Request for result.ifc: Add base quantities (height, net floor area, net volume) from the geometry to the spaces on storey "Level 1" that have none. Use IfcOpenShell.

First a look at what the model holds.

```python
import ifcopenshell
import ifcopenshell.util.element
import ifcopenshell.util.unit

model = ifcopenshell.open("result.ifc")
print(model.schema)
for unit_type in ("LENGTHUNIT", "AREAUNIT", "VOLUMEUNIT"):
    print(unit_type, ifcopenshell.util.unit.calculate_unit_scale(model, unit_type))
storey = next(s for s in model.by_type("IfcBuildingStorey") if s.Name == "Level 1")
spaces = [e for e in ifcopenshell.util.element.get_decomposition(storey) if e.is_a("IfcSpace")]
for e in sorted(spaces, key=lambda e: e.id()):
    print(e.id(), e.is_a(), e.Name, list(ifcopenshell.util.element.get_psets(e, qtos_only=True)), sep=" | ")
```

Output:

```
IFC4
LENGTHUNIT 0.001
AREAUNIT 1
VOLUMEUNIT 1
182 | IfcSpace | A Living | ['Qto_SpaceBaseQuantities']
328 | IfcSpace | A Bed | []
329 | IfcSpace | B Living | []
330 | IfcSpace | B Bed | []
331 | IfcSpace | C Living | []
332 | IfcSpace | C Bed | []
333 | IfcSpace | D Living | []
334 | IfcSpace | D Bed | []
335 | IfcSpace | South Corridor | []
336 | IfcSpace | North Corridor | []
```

```python
import ifcopenshell
import ifcopenshell.api.pset
import ifcopenshell.geom
import ifcopenshell.util.element
import ifcopenshell.util.shape
import ifcopenshell.util.unit

model = ifcopenshell.open("result.ifc")
unit_scale = ifcopenshell.util.unit.calculate_unit_scale(model)
area_scale = ifcopenshell.util.unit.calculate_unit_scale(model, "AREAUNIT")
volume_scale = ifcopenshell.util.unit.calculate_unit_scale(model, "VOLUMEUNIT")
settings = ifcopenshell.geom.settings()

storey = next(s for s in model.by_type("IfcBuildingStorey") if s.Name == "Level 1")
spaces = [e for e in ifcopenshell.util.element.get_decomposition(storey) if e.is_a("IfcSpace")]

for e in sorted(spaces, key=lambda e: e.id()):
    if ifcopenshell.util.element.get_psets(e, qtos_only=True, should_inherit=False):
        continue
    # Geometry comes back in metres, in the element's own axes.
    shape = ifcopenshell.geom.create_shape(settings, e)
    values = {
        "Height": ifcopenshell.util.shape.get_z(shape.geometry) / unit_scale,
        "NetFloorArea": ifcopenshell.util.shape.get_footprint_area(shape.geometry) / area_scale,
        "NetVolume": ifcopenshell.util.shape.get_volume(shape.geometry) / volume_scale,
    }
    qto = ifcopenshell.api.pset.add_qto(model, product=e, name="Qto_SpaceBaseQuantities")
    ifcopenshell.api.pset.edit_qto(model, qto=qto, properties=values)
    print(e.id(), {k: round(v, 3) for k, v in values.items()})

model.write("result-out.ifc")
```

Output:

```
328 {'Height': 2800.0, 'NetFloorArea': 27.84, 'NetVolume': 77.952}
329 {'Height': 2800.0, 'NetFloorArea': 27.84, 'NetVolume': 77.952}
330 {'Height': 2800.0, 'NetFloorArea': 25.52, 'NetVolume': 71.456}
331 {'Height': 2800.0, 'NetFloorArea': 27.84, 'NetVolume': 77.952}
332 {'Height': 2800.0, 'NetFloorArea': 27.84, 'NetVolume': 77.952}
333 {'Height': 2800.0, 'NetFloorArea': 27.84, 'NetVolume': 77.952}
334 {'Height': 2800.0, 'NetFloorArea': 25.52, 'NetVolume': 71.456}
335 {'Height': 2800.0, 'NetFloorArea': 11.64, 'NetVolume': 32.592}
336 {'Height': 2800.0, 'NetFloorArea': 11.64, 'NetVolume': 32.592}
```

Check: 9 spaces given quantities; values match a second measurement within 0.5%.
